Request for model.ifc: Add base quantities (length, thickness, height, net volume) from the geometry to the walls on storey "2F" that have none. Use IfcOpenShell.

First a look at what the model holds.

```python
import ifcopenshell
import ifcopenshell.util.element
import ifcopenshell.util.unit

model = ifcopenshell.open("model.ifc")
print(model.schema)
for unit_type in ("LENGTHUNIT", "AREAUNIT", "VOLUMEUNIT"):
    print(unit_type, ifcopenshell.util.unit.calculate_unit_scale(model, unit_type))
storey = next(s for s in model.by_type("IfcBuildingStorey") if s.Name == "2F")
walls = [e for e in ifcopenshell.util.element.get_decomposition(storey) if e.is_a("IfcWall")]
for e in sorted(walls, key=lambda e: e.id()):
    print(e.id(), e.is_a(), e.Name, list(ifcopenshell.util.element.get_psets(e, qtos_only=True)), sep=" | ")
```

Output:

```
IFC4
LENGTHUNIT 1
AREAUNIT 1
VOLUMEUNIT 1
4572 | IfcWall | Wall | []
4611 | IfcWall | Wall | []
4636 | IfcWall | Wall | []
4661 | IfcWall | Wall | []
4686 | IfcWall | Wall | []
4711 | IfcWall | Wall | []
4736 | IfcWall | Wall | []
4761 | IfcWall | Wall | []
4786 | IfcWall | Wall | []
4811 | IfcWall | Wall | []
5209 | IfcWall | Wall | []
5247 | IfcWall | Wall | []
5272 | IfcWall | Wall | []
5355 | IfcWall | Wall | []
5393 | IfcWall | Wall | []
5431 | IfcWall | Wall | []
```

```python
import ifcopenshell
import ifcopenshell.api.pset
import ifcopenshell.geom
import ifcopenshell.util.element
import ifcopenshell.util.shape
import ifcopenshell.util.unit

model = ifcopenshell.open("model.ifc")
unit_scale = ifcopenshell.util.unit.calculate_unit_scale(model)
volume_scale = ifcopenshell.util.unit.calculate_unit_scale(model, "VOLUMEUNIT")
settings = ifcopenshell.geom.settings()

storey = next(s for s in model.by_type("IfcBuildingStorey") if s.Name == "2F")
walls = [e for e in ifcopenshell.util.element.get_decomposition(storey) if e.is_a("IfcWall")]

for e in sorted(walls, key=lambda e: e.id()):
    if ifcopenshell.util.element.get_psets(e, qtos_only=True, should_inherit=False):
        continue
    # Geometry comes back in metres, in the element's own axes.
    shape = ifcopenshell.geom.create_shape(settings, e)
    values = {
        "Length": ifcopenshell.util.shape.get_x(shape.geometry) / unit_scale,
        "Width": ifcopenshell.util.shape.get_y(shape.geometry) / unit_scale,
        "Height": ifcopenshell.util.shape.get_z(shape.geometry) / unit_scale,
        "NetVolume": ifcopenshell.util.shape.get_volume(shape.geometry) / volume_scale,
    }
    qto = ifcopenshell.api.pset.add_qto(model, product=e, name="Qto_WallBaseQuantities")
    ifcopenshell.api.pset.edit_qto(model, qto=qto, properties=values)
    print(e.id(), {k: round(v, 3) for k, v in values.items()})

model.write("model_v2.ifc")
```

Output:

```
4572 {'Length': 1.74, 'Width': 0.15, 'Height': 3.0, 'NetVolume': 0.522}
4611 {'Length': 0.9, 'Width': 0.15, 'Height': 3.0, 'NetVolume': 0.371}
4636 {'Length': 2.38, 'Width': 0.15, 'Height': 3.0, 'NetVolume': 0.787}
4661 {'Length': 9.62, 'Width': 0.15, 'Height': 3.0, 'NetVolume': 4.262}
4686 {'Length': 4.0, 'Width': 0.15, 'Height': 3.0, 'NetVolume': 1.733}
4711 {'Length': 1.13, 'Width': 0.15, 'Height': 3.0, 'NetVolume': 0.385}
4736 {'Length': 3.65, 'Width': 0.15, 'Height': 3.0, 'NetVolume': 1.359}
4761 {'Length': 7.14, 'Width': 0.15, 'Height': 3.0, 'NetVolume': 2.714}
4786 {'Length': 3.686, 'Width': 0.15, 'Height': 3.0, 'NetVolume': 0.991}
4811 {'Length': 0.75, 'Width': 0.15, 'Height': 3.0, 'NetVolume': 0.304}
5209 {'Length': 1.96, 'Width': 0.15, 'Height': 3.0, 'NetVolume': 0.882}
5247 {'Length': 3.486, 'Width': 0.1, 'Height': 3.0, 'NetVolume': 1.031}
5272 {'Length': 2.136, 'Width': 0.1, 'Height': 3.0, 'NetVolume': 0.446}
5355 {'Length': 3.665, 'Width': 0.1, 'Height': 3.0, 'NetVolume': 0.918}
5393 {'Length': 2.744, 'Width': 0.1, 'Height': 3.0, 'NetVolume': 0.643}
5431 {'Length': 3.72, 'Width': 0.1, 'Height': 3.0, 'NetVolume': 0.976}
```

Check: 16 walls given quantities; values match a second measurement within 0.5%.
